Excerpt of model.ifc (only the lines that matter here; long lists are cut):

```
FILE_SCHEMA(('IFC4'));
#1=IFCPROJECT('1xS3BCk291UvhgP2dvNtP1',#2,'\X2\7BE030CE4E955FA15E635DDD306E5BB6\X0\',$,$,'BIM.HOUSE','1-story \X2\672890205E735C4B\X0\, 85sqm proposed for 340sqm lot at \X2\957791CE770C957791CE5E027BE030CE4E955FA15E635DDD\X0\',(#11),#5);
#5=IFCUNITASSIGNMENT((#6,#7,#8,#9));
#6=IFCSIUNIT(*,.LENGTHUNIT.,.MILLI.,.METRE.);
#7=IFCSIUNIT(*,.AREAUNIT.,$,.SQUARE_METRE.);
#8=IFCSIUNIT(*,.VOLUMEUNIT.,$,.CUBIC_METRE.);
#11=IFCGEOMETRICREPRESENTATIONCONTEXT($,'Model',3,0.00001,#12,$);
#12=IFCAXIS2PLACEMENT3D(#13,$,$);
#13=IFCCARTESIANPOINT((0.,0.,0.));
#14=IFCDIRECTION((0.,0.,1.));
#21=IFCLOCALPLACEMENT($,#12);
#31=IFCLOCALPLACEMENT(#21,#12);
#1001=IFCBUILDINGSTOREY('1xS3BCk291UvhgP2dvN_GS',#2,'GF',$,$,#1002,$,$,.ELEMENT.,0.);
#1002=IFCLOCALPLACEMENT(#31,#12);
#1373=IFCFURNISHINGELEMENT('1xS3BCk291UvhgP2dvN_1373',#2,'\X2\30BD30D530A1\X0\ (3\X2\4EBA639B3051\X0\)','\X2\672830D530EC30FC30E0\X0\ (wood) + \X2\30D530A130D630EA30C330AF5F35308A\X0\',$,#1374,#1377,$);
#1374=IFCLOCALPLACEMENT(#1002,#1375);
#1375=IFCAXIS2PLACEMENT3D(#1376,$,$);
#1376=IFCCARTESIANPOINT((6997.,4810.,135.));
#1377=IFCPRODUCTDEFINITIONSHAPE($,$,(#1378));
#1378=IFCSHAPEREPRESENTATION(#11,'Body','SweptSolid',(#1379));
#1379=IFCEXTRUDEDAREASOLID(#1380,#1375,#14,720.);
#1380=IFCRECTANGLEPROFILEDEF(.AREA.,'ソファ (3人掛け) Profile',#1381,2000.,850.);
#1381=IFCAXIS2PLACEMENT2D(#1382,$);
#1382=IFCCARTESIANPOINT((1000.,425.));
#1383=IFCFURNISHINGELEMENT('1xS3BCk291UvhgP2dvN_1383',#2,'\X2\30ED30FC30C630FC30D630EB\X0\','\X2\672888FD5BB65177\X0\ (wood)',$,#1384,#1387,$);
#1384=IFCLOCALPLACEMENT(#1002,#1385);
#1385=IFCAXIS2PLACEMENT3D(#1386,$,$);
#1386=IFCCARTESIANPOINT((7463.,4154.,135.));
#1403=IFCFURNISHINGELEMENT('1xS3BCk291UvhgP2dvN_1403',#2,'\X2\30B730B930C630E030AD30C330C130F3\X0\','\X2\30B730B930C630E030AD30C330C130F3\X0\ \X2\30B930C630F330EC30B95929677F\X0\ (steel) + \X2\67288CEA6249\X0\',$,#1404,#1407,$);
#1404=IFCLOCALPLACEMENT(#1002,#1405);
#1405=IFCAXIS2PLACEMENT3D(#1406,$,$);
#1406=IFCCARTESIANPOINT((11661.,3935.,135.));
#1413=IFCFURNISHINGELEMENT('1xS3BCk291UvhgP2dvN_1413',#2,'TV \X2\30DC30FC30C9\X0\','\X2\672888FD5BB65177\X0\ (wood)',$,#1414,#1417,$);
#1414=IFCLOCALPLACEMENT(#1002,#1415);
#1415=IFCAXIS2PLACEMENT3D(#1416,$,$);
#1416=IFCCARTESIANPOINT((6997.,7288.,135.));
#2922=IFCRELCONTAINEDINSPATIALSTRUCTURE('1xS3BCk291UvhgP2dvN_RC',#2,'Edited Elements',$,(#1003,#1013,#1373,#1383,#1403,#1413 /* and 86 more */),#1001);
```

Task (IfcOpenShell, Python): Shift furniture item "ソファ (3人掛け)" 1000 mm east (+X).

```python
import ifcopenshell
import ifcopenshell.api.geometry
import ifcopenshell.util.placement
import ifcopenshell.util.unit

model = ifcopenshell.open("model.ifc")
unit_scale = ifcopenshell.util.unit.calculate_unit_scale(model)

item = model.by_guid("1xS3BCk291UvhgP2dvN_1373")
matrix = ifcopenshell.util.placement.get_local_placement(item.ObjectPlacement)
matrix[0, 3] += 1 / unit_scale
ifcopenshell.api.geometry.edit_object_placement(model, product=item, matrix=matrix, is_si=False)

print(ifcopenshell.util.placement.get_local_placement(item.ObjectPlacement).round(3) + 0.0)

model.write("model_edited.ifc")
```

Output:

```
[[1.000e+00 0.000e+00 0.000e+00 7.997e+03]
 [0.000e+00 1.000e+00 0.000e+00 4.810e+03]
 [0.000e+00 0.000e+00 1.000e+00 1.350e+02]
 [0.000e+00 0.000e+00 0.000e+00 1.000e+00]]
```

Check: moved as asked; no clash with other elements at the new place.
